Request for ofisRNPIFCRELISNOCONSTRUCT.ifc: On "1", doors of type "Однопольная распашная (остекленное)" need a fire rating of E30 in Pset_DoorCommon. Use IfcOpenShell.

First a look at what the model holds.

```python
import ifcopenshell
import ifcopenshell.util.element

model = ifcopenshell.open("ofisRNPIFCRELISNOCONSTRUCT.ifc")
print(model.schema)
storey = next(s for s in model.by_type("IfcBuildingStorey") if s.Name == "1")
doors = [e for e in ifcopenshell.util.element.get_decomposition(storey) if e.is_a("IfcDoor")]
seen = {}
for e in doors:
    element_type = ifcopenshell.util.element.get_type(e)
    key = (element_type.Name if element_type != e and element_type else None, ifcopenshell.util.element.get_pset(e, "Pset_DoorCommon", "FireRating"))
    seen[key] = seen.get(key, 0) + 1
for (name, value), count in sorted(seen.items(), key=str):
    print(count, "x", name, "|", value)
```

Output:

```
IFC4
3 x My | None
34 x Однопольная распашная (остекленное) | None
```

```python
import ifcopenshell
import ifcopenshell.api.pset
import ifcopenshell.util.element

model = ifcopenshell.open("ofisRNPIFCRELISNOCONSTRUCT.ifc")

storey = next(s for s in model.by_type("IfcBuildingStorey") if s.Name == "1")
doors = [e for e in ifcopenshell.util.element.get_decomposition(storey) if e.is_a("IfcDoor")]

count = 0
for e in doors:
    element_type = ifcopenshell.util.element.get_type(e)
    if element_type in (None, e) or element_type.Name != "Однопольная распашная (остекленное)":
        continue
    # add_pset returns the element's existing set when there is one.
    pset = ifcopenshell.api.pset.add_pset(model, product=e, name="Pset_DoorCommon")
    ifcopenshell.api.pset.edit_pset(model, pset=pset, properties={"FireRating": "E30"})
    count += 1

print(count, "doors updated")

model.write("ofisRNPIFCRELISNOCONSTRUCT_v2.ifc")
```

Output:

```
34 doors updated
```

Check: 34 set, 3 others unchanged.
